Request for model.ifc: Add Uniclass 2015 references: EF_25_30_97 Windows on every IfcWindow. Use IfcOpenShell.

First a look at what the model holds.

```python
import ifcopenshell

model = ifcopenshell.open("model.ifc")
print(model.schema)
print("classifications:", [c.Name for c in model.by_type("IfcClassification")])
for ifc_class in ("IfcDoor", "IfcRoof", "IfcStair", "IfcWall", "IfcWindow"):
    print(ifc_class, len(model.by_type(ifc_class)))
```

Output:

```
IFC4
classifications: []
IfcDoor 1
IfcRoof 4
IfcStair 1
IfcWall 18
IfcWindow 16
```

```python
import ifcopenshell
import ifcopenshell.api.classification

model = ifcopenshell.open("model.ifc")

system = ifcopenshell.api.classification.add_classification(model, classification="Uniclass 2015")

codes = {
    "IfcWindow": ("EF_25_30_97", "Windows"),
}
for ifc_class, (code, name) in codes.items():
    products = model.by_type(ifc_class)
    ifcopenshell.api.classification.add_reference(
        model, products=products, classification=system, identification=code, name=name
    )
    print(code, len(products))

model.write("model_updated.ifc")
```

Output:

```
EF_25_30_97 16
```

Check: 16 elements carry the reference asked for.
